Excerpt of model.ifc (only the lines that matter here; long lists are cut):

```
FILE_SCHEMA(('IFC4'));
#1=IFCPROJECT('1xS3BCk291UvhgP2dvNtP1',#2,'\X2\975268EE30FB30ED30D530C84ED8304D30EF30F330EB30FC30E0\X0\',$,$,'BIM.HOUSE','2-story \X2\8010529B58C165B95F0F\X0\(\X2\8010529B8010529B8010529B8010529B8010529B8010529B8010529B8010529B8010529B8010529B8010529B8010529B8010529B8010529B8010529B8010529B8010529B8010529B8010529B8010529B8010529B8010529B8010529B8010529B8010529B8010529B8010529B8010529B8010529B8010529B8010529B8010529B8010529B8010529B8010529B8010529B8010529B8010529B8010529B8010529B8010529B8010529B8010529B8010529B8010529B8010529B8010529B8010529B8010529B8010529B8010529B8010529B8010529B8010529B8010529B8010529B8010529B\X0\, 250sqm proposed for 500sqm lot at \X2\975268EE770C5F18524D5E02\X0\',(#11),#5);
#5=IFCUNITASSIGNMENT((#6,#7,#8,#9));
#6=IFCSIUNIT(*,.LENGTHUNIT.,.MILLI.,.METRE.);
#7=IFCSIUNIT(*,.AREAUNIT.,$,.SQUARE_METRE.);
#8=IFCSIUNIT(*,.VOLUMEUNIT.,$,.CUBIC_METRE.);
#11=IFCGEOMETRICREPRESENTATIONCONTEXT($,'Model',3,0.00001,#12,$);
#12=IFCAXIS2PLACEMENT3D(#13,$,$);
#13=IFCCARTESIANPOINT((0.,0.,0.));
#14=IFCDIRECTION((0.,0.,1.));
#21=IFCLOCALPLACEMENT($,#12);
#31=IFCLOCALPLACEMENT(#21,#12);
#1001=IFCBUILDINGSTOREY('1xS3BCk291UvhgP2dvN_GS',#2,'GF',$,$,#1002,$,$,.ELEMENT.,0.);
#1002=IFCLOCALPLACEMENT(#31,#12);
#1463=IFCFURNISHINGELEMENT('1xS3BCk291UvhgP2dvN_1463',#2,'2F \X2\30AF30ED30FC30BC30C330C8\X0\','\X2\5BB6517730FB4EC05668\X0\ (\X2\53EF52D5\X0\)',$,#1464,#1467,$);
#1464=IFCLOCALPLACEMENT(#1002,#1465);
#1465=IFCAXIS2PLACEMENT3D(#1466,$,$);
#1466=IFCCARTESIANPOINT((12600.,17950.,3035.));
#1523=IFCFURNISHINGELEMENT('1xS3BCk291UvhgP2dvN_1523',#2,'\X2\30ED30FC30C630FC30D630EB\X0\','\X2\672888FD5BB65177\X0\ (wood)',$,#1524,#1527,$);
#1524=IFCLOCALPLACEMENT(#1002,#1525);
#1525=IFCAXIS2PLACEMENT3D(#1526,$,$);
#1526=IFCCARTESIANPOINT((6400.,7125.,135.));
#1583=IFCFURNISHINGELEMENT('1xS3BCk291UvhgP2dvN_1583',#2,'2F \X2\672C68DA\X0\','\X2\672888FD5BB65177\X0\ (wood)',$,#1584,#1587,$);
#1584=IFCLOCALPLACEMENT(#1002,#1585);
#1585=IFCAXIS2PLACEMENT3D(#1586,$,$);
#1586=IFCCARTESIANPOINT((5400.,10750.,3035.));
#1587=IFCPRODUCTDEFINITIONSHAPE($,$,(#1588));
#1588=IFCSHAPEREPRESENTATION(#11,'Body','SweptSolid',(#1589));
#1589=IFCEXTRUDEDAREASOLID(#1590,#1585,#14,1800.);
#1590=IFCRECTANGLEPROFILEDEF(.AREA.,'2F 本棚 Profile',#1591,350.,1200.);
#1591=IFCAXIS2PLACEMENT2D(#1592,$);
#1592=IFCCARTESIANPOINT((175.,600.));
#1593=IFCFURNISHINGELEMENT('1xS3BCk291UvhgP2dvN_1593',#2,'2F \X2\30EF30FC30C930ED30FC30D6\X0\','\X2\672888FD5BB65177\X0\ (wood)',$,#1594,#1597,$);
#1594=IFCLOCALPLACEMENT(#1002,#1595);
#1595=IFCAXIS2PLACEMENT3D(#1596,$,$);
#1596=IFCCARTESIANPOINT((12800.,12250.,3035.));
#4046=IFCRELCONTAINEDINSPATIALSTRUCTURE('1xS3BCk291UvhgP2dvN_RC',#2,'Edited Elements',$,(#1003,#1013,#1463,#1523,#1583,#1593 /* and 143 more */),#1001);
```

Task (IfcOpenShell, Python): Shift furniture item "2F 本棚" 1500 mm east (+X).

```python
import ifcopenshell
import ifcopenshell.api.geometry
import ifcopenshell.util.placement
import ifcopenshell.util.unit

model = ifcopenshell.open("model.ifc")
unit_scale = ifcopenshell.util.unit.calculate_unit_scale(model)

item = model.by_id(1583)
matrix = ifcopenshell.util.placement.get_local_placement(item.ObjectPlacement)
matrix[0, 3] += 1.5 / unit_scale
ifcopenshell.api.geometry.edit_object_placement(model, product=item, matrix=matrix, is_si=False)

print(ifcopenshell.util.placement.get_local_placement(item.ObjectPlacement).round(3) + 0.0)

model.write("model_rev.ifc")
```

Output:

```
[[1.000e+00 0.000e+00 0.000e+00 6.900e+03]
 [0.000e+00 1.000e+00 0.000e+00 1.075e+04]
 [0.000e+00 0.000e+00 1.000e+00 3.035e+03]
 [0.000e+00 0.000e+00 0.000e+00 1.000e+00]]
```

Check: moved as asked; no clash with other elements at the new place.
